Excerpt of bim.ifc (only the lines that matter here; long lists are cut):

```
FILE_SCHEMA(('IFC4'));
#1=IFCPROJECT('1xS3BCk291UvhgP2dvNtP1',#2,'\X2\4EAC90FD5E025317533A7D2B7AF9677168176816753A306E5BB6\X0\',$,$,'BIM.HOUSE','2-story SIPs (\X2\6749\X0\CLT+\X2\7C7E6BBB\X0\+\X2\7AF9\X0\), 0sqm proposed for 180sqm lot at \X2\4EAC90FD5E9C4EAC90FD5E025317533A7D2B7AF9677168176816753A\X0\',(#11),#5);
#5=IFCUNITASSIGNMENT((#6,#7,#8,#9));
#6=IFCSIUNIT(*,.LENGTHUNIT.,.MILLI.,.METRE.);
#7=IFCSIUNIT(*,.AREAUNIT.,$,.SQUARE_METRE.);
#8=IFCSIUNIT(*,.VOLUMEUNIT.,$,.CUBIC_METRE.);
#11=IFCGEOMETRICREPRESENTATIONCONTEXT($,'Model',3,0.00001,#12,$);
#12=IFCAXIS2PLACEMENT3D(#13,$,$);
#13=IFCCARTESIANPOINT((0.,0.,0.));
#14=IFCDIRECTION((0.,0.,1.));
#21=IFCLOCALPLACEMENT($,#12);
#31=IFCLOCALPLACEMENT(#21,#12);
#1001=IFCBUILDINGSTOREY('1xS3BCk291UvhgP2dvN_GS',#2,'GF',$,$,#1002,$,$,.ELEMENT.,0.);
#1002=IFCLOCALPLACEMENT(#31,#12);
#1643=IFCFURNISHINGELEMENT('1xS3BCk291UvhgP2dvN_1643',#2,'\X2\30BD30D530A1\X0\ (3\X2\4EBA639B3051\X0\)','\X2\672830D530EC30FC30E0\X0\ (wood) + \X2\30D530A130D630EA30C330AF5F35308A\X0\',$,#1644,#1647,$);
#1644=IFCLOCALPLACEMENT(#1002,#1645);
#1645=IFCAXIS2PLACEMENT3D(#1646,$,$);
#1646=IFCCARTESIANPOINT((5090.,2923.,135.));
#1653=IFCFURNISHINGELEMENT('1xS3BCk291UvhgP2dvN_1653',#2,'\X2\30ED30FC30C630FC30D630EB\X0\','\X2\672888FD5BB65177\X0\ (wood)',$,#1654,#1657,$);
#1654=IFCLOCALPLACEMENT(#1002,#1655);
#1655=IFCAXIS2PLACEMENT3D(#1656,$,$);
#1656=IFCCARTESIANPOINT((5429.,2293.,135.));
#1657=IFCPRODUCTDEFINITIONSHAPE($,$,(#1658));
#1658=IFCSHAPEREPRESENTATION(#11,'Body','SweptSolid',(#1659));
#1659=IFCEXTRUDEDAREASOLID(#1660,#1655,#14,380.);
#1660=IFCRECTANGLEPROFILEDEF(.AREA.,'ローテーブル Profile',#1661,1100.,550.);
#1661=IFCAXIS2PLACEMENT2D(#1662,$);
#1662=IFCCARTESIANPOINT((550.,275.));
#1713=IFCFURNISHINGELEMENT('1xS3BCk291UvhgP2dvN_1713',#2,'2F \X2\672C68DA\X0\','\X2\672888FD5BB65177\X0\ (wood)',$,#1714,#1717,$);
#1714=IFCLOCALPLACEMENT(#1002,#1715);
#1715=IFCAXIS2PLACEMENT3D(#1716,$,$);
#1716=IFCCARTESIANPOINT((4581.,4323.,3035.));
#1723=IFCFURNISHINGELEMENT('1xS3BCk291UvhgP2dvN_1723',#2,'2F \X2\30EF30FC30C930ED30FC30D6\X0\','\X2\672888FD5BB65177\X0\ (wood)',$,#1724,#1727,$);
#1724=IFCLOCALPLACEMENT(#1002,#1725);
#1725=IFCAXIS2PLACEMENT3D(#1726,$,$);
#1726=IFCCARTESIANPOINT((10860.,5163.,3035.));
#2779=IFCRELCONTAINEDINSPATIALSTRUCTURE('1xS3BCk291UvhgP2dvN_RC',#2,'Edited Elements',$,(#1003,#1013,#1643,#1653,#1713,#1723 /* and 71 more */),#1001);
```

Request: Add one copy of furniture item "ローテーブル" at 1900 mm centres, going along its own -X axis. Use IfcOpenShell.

```python
import ifcopenshell
import ifcopenshell.api.geometry
import ifcopenshell.api.root
import ifcopenshell.util.element
import ifcopenshell.util.placement

model = ifcopenshell.open("bim.ifc")


def reuse_history(source, copy):
    """copy_class also copies each property set's owner history, people and application; keep the originals."""
    for rel in copy.IsDefinedBy:
        if rel.is_a("IfcRelDefinesByProperties") and (history := rel.RelatingPropertyDefinition.OwnerHistory):
            rel.RelatingPropertyDefinition.OwnerHistory = source.OwnerHistory
            ifcopenshell.util.element.remove_deep2(model, history)


source = model.by_guid("1xS3BCk291UvhgP2dvN_1653")
base = ifcopenshell.util.placement.get_local_placement(source.ObjectPlacement)
step = -base[:3, 0] * 1900.0

for i in range(1, 2):
    copy = ifcopenshell.api.root.copy_class(model, product=source)
    copy.Representation = ifcopenshell.util.element.copy_deep(
        model, source.Representation, exclude=["IfcGeometricRepresentationContext", "IfcRepresentationMap"]
    )
    reuse_history(source, copy)
    matrix = base.copy()
    matrix[:3, 3] += i * step
    print("added at", matrix[:3, 3].round(3) + 0.0)
    ifcopenshell.api.geometry.edit_object_placement(model, product=copy, matrix=matrix, is_si=False)

model.write("bim-out.ifc")
```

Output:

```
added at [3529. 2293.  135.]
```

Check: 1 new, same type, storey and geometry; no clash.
